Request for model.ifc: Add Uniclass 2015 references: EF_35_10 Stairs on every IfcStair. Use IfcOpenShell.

First a look at what the model holds.

```python
import ifcopenshell

model = ifcopenshell.open("model.ifc")
print(model.schema)
print("classifications:", [c.Name for c in model.by_type("IfcClassification")])
for ifc_class in ("IfcDoor", "IfcRoof", "IfcStair", "IfcWall", "IfcWindow"):
    print(ifc_class, len(model.by_type(ifc_class)))
```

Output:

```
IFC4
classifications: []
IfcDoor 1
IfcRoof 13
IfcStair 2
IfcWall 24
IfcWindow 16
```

```python
import ifcopenshell
import ifcopenshell.api.classification

model = ifcopenshell.open("model.ifc")

system = ifcopenshell.api.classification.add_classification(model, classification="Uniclass 2015")

codes = {
    "IfcStair": ("EF_35_10", "Stairs"),
}
for ifc_class, (code, name) in codes.items():
    products = model.by_type(ifc_class)
    ifcopenshell.api.classification.add_reference(
        model, products=products, classification=system, identification=code, name=name
    )
    print(code, len(products))

model.write("model-out.ifc")
```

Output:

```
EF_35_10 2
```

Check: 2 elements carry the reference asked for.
